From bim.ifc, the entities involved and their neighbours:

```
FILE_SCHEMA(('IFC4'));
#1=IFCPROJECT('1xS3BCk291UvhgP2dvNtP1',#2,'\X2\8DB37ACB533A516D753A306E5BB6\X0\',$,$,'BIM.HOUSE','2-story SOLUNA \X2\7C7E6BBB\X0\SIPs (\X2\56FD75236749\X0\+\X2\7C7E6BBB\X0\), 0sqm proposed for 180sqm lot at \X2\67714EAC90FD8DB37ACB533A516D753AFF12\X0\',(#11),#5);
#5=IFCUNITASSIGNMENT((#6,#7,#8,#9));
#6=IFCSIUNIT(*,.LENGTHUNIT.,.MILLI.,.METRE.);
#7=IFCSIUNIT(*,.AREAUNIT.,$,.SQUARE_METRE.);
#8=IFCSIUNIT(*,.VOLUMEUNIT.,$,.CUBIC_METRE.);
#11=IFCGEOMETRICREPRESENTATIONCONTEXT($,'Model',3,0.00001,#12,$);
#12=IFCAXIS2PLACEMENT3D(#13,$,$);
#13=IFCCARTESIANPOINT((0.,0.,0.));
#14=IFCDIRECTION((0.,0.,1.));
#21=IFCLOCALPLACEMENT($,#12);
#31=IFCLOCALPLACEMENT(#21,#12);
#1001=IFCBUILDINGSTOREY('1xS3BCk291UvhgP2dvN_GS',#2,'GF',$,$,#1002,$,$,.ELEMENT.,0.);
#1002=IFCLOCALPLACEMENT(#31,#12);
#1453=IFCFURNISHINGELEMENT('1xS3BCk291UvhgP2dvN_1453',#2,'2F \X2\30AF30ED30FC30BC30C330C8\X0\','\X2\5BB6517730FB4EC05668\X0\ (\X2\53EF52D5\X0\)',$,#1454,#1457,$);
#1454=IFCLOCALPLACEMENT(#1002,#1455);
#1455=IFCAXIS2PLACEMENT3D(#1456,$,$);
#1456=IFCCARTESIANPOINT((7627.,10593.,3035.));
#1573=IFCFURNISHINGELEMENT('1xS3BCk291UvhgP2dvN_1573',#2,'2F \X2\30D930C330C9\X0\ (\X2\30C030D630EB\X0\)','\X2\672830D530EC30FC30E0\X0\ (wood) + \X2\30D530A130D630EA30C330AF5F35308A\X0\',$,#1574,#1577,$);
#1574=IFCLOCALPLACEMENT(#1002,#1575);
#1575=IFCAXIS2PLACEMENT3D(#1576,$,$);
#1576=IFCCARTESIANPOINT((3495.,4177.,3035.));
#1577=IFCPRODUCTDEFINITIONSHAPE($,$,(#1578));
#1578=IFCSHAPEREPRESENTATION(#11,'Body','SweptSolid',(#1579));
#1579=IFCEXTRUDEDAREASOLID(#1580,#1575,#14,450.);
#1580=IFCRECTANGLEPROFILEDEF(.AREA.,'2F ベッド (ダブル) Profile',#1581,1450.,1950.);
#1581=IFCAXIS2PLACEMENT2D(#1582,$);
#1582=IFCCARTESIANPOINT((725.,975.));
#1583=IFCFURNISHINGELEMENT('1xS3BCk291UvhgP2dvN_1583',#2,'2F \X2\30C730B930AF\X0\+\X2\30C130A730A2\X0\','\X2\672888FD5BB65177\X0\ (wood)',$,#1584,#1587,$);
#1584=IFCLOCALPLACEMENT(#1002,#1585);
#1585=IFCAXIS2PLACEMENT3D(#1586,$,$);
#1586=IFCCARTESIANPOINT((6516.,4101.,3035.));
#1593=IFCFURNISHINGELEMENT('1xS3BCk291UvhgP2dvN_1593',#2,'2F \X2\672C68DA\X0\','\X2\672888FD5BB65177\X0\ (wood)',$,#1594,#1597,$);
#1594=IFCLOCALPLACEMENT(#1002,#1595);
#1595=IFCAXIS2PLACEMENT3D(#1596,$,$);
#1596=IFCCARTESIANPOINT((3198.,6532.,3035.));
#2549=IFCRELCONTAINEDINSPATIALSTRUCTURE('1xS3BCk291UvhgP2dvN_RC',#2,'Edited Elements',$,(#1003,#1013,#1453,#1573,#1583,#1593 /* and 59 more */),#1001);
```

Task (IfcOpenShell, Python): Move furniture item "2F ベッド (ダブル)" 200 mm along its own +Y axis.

```python
import ifcopenshell
import ifcopenshell.api.geometry
import ifcopenshell.util.placement

model = ifcopenshell.open("bim.ifc")

item = model.by_guid("1xS3BCk291UvhgP2dvN_1573")
matrix = ifcopenshell.util.placement.get_local_placement(item.ObjectPlacement)
matrix[:3, 3] += matrix[:3, 1] * 200.0
ifcopenshell.api.geometry.edit_object_placement(model, product=item, matrix=matrix, is_si=False)

print(ifcopenshell.util.placement.get_local_placement(item.ObjectPlacement).round(3) + 0.0)

model.write("bim_rev.ifc")
```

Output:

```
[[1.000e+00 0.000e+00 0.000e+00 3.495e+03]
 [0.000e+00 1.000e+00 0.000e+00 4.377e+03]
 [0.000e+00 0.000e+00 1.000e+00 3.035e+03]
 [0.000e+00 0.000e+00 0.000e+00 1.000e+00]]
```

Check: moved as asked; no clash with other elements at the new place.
